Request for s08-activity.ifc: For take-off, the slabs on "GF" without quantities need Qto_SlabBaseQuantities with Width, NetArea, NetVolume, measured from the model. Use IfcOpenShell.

First a look at what the model holds.

```python
import ifcopenshell
import ifcopenshell.util.element
import ifcopenshell.util.unit

model = ifcopenshell.open("s08-activity.ifc")
print(model.schema)
for unit_type in ("LENGTHUNIT", "AREAUNIT", "VOLUMEUNIT"):
    print(unit_type, ifcopenshell.util.unit.calculate_unit_scale(model, unit_type))
storey = next(s for s in model.by_type("IfcBuildingStorey") if s.Name == "GF")
slabs = [e for e in ifcopenshell.util.element.get_decomposition(storey) if e.is_a("IfcSlab")]
for e in sorted(slabs, key=lambda e: e.id()):
    print(e.id(), e.is_a(), e.Name, list(ifcopenshell.util.element.get_psets(e, qtos_only=True)), sep=" | ")
```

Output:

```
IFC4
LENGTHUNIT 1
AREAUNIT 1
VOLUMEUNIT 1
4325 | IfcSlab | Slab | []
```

```python
import ifcopenshell
import ifcopenshell.api.pset
import ifcopenshell.geom
import ifcopenshell.util.element
import ifcopenshell.util.shape
import ifcopenshell.util.unit

model = ifcopenshell.open("s08-activity.ifc")
unit_scale = ifcopenshell.util.unit.calculate_unit_scale(model)
area_scale = ifcopenshell.util.unit.calculate_unit_scale(model, "AREAUNIT")
volume_scale = ifcopenshell.util.unit.calculate_unit_scale(model, "VOLUMEUNIT")
settings = ifcopenshell.geom.settings()

storey = next(s for s in model.by_type("IfcBuildingStorey") if s.Name == "GF")
slabs = [e for e in ifcopenshell.util.element.get_decomposition(storey) if e.is_a("IfcSlab")]

for e in sorted(slabs, key=lambda e: e.id()):
    if ifcopenshell.util.element.get_psets(e, qtos_only=True, should_inherit=False):
        continue
    # Geometry comes back in metres, in the element's own axes.
    shape = ifcopenshell.geom.create_shape(settings, e)
    values = {
        "Width": ifcopenshell.util.shape.get_z(shape.geometry) / unit_scale,
        "NetArea": ifcopenshell.util.shape.get_footprint_area(shape.geometry) / area_scale,
        "NetVolume": ifcopenshell.util.shape.get_volume(shape.geometry) / volume_scale,
    }
    qto = ifcopenshell.api.pset.add_qto(model, product=e, name="Qto_SlabBaseQuantities")
    ifcopenshell.api.pset.edit_qto(model, qto=qto, properties=values)
    print(e.id(), {k: round(v, 3) for k, v in values.items()})

model.write("s08-activity_edited.ifc")
```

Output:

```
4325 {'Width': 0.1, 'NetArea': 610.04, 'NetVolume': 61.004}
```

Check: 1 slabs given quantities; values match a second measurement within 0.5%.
